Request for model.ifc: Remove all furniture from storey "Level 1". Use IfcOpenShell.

First a look at what the model holds.

```python
import ifcopenshell
import ifcopenshell.util.element

model = ifcopenshell.open("model.ifc")
print(model.schema)
storey = next(s for s in model.by_type("IfcBuildingStorey") if s.Name == "Level 1")
furniture = [e for e in ifcopenshell.util.element.get_decomposition(storey) if e.is_a("IfcFurnishingElement")]
seen = {}
for e in furniture:
    element_type = ifcopenshell.util.element.get_type(e)
    name = element_type.Name if element_type not in (None, e) else None
    seen[name] = seen.get(name, 0) + 1
for name, count in sorted(seen.items(), key=str):
    print(count, "x", name)
```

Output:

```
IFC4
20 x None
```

```python
import ifcopenshell
import ifcopenshell.api.root
import ifcopenshell.util.element

model = ifcopenshell.open("model.ifc")

storey = next(s for s in model.by_type("IfcBuildingStorey") if s.Name == "Level 1")
furniture = [e for e in ifcopenshell.util.element.get_decomposition(storey) if e.is_a("IfcFurnishingElement")]

for e in furniture:
    ifcopenshell.api.root.remove_product(model, product=e)
print(len(furniture), "removed")

model.write("model_updated.ifc")
```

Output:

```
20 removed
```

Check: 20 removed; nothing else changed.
